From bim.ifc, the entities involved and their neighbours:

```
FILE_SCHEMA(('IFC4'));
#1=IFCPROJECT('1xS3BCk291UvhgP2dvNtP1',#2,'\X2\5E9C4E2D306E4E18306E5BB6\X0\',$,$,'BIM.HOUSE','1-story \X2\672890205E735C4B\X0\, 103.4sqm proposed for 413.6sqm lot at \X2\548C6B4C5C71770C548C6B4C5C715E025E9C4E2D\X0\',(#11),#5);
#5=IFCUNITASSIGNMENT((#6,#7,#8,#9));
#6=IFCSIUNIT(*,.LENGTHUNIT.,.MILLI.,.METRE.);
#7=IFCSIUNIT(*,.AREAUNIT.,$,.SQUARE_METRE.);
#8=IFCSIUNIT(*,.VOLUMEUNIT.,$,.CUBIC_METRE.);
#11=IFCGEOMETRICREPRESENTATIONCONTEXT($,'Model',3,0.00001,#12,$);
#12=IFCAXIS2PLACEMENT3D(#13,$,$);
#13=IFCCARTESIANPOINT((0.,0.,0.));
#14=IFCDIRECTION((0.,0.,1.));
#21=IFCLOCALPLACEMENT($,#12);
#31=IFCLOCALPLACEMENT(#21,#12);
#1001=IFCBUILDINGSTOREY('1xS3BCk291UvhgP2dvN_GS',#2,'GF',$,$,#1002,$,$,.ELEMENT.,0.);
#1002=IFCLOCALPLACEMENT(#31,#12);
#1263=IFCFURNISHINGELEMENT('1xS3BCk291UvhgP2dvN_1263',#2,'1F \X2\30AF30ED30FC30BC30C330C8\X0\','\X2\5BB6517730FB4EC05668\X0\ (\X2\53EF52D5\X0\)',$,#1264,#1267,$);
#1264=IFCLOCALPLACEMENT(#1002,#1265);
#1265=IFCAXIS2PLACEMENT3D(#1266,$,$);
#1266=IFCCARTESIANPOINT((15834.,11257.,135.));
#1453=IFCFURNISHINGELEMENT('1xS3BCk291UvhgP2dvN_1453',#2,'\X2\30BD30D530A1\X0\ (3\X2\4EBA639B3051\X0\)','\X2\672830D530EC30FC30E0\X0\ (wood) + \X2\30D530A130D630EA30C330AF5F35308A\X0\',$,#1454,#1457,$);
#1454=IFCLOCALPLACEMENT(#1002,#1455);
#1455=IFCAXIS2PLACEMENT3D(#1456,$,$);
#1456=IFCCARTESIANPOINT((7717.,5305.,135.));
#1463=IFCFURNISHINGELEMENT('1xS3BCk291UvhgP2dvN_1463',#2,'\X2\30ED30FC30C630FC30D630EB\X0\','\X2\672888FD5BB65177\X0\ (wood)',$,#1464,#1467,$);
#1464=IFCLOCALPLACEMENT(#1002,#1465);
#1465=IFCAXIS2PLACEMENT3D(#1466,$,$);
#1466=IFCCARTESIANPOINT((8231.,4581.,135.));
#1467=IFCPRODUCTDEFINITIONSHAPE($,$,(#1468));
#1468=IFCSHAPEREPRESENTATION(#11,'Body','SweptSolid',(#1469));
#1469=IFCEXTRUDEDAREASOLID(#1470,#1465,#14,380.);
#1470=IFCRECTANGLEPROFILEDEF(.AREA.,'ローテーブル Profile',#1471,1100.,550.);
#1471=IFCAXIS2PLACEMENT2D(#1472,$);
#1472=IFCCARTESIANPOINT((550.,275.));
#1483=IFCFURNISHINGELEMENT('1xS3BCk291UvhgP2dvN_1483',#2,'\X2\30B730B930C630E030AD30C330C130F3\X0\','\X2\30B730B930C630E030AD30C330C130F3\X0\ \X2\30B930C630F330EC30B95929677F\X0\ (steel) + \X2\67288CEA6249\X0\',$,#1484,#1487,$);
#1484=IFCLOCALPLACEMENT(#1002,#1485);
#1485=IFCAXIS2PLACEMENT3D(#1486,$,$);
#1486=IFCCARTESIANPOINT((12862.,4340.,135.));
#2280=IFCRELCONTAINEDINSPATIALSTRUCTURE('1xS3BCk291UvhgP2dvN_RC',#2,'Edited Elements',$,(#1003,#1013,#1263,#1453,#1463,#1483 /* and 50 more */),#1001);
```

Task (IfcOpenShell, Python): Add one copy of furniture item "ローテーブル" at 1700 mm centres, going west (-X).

```python
import numpy as np
import ifcopenshell
import ifcopenshell.api.geometry
import ifcopenshell.api.root
import ifcopenshell.util.element
import ifcopenshell.util.placement
import ifcopenshell.util.unit

model = ifcopenshell.open("bim.ifc")
unit_scale = ifcopenshell.util.unit.calculate_unit_scale(model)


def reuse_history(source, copy):
    """copy_class also copies each property set's owner history, people and application; keep the originals."""
    for rel in copy.IsDefinedBy:
        if rel.is_a("IfcRelDefinesByProperties") and (history := rel.RelatingPropertyDefinition.OwnerHistory):
            rel.RelatingPropertyDefinition.OwnerHistory = source.OwnerHistory
            ifcopenshell.util.element.remove_deep2(model, history)


source = model.by_guid("1xS3BCk291UvhgP2dvN_1463")
base = ifcopenshell.util.placement.get_local_placement(source.ObjectPlacement)
step = np.array([-1.0, 0.0, 0.0]) * 1.7 / unit_scale

for i in range(1, 2):
    copy = ifcopenshell.api.root.copy_class(model, product=source)
    copy.Representation = ifcopenshell.util.element.copy_deep(
        model, source.Representation, exclude=["IfcGeometricRepresentationContext", "IfcRepresentationMap"]
    )
    reuse_history(source, copy)
    matrix = base.copy()
    matrix[:3, 3] += i * step
    print("added at", matrix[:3, 3].round(3) + 0.0)
    ifcopenshell.api.geometry.edit_object_placement(model, product=copy, matrix=matrix, is_si=False)

model.write("bim_v2.ifc")
```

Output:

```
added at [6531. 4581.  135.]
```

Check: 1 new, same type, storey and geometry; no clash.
